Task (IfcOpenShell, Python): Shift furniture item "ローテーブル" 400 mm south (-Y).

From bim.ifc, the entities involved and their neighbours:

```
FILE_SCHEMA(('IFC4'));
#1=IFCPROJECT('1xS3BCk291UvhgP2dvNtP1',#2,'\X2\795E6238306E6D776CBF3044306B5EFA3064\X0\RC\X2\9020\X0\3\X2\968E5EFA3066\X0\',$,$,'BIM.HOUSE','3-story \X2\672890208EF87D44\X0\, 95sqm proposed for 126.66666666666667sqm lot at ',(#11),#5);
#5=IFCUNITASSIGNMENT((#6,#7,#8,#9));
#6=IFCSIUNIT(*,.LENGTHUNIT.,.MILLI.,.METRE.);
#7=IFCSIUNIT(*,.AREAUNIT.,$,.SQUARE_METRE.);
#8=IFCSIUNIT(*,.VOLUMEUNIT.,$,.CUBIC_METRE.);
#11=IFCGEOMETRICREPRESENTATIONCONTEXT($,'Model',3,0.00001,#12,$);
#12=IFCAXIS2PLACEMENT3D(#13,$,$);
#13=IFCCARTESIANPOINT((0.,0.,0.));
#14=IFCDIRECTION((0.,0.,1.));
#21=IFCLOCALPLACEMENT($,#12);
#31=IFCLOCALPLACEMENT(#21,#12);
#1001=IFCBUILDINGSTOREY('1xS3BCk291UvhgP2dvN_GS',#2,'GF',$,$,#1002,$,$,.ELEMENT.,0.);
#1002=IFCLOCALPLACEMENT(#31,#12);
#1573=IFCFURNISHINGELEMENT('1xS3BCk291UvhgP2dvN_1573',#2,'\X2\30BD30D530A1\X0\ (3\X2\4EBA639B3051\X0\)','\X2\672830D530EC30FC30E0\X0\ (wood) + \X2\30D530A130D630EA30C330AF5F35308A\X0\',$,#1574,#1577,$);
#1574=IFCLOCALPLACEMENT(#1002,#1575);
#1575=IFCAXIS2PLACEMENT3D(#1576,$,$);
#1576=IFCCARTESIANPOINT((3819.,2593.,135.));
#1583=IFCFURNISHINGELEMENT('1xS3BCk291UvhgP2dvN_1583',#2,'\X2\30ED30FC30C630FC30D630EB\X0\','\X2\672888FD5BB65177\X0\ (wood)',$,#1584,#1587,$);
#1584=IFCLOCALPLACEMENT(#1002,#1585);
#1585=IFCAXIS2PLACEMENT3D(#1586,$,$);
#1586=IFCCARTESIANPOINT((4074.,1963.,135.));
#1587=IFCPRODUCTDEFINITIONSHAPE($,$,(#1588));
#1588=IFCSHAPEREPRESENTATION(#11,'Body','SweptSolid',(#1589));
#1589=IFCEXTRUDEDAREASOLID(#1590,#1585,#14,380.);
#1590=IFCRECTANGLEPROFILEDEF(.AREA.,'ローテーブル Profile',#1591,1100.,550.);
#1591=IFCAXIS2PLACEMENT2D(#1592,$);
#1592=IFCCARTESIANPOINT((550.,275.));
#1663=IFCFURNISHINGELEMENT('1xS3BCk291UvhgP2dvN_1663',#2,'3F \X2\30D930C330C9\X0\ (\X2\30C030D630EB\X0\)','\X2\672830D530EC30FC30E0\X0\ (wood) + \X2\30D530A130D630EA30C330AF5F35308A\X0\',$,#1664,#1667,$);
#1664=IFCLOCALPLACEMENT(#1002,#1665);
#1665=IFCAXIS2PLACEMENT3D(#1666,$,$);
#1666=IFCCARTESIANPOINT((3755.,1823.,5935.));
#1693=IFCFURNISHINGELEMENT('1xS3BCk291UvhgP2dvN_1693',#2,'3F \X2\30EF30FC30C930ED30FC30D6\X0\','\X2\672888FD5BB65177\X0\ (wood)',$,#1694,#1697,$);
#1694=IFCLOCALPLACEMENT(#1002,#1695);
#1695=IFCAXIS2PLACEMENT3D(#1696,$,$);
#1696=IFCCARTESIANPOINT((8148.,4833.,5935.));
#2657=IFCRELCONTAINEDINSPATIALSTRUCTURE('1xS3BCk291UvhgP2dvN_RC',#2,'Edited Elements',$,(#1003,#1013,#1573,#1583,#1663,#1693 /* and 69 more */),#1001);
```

```python
import ifcopenshell
import ifcopenshell.api.geometry
import ifcopenshell.util.placement
import ifcopenshell.util.unit

model = ifcopenshell.open("bim.ifc")
unit_scale = ifcopenshell.util.unit.calculate_unit_scale(model)

item = model.by_id(1583)
matrix = ifcopenshell.util.placement.get_local_placement(item.ObjectPlacement)
matrix[1, 3] -= 0.4 / unit_scale
ifcopenshell.api.geometry.edit_object_placement(model, product=item, matrix=matrix, is_si=False)

print(ifcopenshell.util.placement.get_local_placement(item.ObjectPlacement).round(3) + 0.0)

model.write("bim-out.ifc")
```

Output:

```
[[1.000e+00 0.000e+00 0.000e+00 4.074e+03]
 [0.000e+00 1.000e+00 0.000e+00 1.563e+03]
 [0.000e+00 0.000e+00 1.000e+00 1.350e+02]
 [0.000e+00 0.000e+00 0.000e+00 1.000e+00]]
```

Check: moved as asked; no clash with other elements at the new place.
